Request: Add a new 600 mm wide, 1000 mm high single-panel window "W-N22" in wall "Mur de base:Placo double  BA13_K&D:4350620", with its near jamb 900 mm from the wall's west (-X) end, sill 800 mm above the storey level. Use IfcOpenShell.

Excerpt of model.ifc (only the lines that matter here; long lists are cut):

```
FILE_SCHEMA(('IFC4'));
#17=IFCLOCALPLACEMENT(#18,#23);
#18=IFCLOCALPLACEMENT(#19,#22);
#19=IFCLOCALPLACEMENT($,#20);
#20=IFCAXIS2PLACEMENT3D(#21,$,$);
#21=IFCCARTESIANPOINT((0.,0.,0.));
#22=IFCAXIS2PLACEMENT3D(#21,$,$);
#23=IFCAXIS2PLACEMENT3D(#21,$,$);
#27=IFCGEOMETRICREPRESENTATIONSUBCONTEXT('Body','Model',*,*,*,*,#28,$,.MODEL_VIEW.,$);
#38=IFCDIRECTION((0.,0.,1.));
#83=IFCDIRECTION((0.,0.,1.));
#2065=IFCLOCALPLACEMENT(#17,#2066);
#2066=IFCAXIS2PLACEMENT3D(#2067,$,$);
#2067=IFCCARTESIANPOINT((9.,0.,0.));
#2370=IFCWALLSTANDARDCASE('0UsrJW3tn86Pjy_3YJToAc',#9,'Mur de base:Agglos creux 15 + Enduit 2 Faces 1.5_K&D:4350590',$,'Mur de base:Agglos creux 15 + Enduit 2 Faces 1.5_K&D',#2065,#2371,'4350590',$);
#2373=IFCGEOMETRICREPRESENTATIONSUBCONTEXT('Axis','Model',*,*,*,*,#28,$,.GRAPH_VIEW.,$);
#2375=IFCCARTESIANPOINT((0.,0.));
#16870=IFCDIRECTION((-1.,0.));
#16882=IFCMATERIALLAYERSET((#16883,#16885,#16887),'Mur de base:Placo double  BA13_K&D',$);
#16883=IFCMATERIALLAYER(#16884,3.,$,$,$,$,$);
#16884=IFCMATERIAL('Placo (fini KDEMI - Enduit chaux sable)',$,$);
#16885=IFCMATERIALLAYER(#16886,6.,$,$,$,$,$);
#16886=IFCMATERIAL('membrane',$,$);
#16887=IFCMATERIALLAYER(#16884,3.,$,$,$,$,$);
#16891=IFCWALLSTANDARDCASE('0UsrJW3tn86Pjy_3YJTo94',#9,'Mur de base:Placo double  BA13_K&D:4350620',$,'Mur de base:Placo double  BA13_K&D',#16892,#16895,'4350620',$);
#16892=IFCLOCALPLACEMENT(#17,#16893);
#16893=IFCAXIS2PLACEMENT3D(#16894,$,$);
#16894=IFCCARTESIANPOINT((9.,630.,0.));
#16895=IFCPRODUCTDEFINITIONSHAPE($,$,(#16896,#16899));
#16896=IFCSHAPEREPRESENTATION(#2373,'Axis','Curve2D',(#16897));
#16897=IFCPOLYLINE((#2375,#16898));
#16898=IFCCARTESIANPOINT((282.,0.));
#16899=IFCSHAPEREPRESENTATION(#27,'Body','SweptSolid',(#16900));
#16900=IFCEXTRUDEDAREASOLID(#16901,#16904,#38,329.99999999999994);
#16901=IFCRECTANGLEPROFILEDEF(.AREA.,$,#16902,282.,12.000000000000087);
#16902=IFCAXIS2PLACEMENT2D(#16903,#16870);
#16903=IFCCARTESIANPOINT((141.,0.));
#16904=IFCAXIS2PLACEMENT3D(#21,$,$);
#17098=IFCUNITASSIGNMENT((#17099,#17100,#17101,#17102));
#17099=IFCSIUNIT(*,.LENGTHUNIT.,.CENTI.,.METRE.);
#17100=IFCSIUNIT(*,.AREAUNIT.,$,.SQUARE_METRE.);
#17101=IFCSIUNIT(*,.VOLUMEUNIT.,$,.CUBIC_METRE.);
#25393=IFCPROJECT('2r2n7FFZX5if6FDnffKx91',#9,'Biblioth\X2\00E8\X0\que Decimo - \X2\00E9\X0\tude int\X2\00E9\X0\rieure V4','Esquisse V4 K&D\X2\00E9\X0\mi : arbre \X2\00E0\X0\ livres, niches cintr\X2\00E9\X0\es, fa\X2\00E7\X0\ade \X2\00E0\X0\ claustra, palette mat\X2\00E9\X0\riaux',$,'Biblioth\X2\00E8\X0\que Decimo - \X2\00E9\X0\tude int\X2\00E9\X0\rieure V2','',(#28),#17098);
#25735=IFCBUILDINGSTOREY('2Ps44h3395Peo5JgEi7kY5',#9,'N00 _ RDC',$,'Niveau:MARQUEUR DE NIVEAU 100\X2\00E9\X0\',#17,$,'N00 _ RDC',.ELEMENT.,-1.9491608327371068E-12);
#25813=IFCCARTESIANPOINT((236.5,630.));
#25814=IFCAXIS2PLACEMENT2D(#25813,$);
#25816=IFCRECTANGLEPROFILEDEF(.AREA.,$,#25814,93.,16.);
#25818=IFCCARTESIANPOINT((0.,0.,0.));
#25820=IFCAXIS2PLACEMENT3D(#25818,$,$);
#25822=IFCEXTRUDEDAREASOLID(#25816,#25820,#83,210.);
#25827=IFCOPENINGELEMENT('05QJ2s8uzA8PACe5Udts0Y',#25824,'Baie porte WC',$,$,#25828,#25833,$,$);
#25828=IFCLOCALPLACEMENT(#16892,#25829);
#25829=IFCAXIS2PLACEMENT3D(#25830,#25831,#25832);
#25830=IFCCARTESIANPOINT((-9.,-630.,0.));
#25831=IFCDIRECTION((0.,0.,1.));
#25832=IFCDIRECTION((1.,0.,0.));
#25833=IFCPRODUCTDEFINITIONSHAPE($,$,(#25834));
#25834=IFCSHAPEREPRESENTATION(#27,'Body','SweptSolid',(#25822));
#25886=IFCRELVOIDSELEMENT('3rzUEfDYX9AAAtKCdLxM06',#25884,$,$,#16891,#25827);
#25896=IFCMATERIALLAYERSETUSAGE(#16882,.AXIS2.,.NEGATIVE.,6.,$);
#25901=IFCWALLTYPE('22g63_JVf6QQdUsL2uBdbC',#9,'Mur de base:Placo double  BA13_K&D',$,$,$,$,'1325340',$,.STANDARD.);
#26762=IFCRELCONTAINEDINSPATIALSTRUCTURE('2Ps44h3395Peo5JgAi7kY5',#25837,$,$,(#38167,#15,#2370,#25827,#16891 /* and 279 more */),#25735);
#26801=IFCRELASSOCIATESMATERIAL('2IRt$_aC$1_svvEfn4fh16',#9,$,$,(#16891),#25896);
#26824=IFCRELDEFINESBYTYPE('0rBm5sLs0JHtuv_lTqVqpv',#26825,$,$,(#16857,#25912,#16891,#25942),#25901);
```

```python
import numpy as np
import ifcopenshell
import ifcopenshell.api.feature
import ifcopenshell.api.geometry
import ifcopenshell.api.root
import ifcopenshell.api.spatial
import ifcopenshell.geom
import ifcopenshell.util.element
import ifcopenshell.util.placement
import ifcopenshell.util.representation
import ifcopenshell.util.shape
import ifcopenshell.util.unit

model = ifcopenshell.open("model.ifc")
unit_scale = ifcopenshell.util.unit.calculate_unit_scale(model)
settings = ifcopenshell.geom.settings()


def volume(element):
    """Net volume in cubic metres, openings subtracted."""
    shape = ifcopenshell.geom.create_shape(settings, element)
    return ifcopenshell.util.shape.get_volume(shape.geometry)


wall = model.by_guid("0UsrJW3tn86Pjy_3YJTo94")
storey = ifcopenshell.util.element.get_container(wall, ifc_class="IfcBuildingStorey")
context = ifcopenshell.util.representation.get_context(model, "Model", "Body", "MODEL_VIEW")
before = volume(wall)

width, height, from_end, sill = 0.6, 1, 0.9, 0.8  # metres

# The wall runs along its own X axis, and the end named is its -X end.
wall_shape = ifcopenshell.geom.create_shape(settings, wall)
x, y, z = ifcopenshell.util.shape.get_vertices(wall_shape.geometry).T
start = x.min() + from_end
face, thickness = float(y.min()), float(y.max() - y.min())
wall_matrix = ifcopenshell.util.placement.get_local_placement(wall.ObjectPlacement)
level = ifcopenshell.util.placement.get_local_placement(storey.ObjectPlacement)[2, 3]


def in_wall(x, y):
    """Placement at x, y metres in the wall's axes, at sill height."""
    matrix = wall_matrix.copy()
    matrix[:, 3] = wall_matrix @ np.array([x / unit_scale, y / unit_scale, 0.0, 1.0])
    matrix[2, 3] = level + sill / unit_scale
    return matrix


# Opening: a box that overshoots both wall faces by 50 mm.
opening = ifcopenshell.api.root.create_entity(model, ifc_class="IfcOpeningElement", predefined_type="OPENING")
box = ifcopenshell.api.geometry.add_wall_representation(
    model, context=context, length=width, height=height, thickness=thickness + 0.1
)
ifcopenshell.api.geometry.assign_representation(model, product=opening, representation=box)
ifcopenshell.api.geometry.edit_object_placement(model, product=opening, matrix=in_wall(start, face - 0.05), is_si=False)
ifcopenshell.api.feature.add_feature(model, feature=opening, element=wall)

window = ifcopenshell.api.root.create_entity(model, ifc_class="IfcWindow", name="W-N22", predefined_type="WINDOW")
window.OverallWidth, window.OverallHeight = width / unit_scale, height / unit_scale
window.PartitioningType = "SINGLE_PANEL"
body = ifcopenshell.api.geometry.add_window_representation(
    model,
    context=context,
    overall_width=window.OverallWidth,
    overall_height=window.OverallHeight,
    partition_type="SINGLE_PANEL",
)
ifcopenshell.api.geometry.assign_representation(model, product=window, representation=body)
ifcopenshell.api.spatial.assign_container(model, products=[window], relating_structure=storey)
ifcopenshell.api.feature.add_filling(model, opening=opening, element=window)

# Centre the window in the wall's thickness.
ifcopenshell.api.geometry.edit_object_placement(model, product=window, matrix=in_wall(start, face), is_si=False)
window_shape = ifcopenshell.geom.create_shape(settings, window)
depth = ifcopenshell.util.shape.get_vertices(window_shape.geometry)[:, 1]
offset = face + thickness / 2 - (depth.min() + depth.max()) / 2
ifcopenshell.api.geometry.edit_object_placement(model, product=window, matrix=in_wall(start, offset), is_si=False)

after = volume(wall)

print(f"wall volume {before:.3f} -> {after:.3f} m3")

model.write("model_updated.ifc")
```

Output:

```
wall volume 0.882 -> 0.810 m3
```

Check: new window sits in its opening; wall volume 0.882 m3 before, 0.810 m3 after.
